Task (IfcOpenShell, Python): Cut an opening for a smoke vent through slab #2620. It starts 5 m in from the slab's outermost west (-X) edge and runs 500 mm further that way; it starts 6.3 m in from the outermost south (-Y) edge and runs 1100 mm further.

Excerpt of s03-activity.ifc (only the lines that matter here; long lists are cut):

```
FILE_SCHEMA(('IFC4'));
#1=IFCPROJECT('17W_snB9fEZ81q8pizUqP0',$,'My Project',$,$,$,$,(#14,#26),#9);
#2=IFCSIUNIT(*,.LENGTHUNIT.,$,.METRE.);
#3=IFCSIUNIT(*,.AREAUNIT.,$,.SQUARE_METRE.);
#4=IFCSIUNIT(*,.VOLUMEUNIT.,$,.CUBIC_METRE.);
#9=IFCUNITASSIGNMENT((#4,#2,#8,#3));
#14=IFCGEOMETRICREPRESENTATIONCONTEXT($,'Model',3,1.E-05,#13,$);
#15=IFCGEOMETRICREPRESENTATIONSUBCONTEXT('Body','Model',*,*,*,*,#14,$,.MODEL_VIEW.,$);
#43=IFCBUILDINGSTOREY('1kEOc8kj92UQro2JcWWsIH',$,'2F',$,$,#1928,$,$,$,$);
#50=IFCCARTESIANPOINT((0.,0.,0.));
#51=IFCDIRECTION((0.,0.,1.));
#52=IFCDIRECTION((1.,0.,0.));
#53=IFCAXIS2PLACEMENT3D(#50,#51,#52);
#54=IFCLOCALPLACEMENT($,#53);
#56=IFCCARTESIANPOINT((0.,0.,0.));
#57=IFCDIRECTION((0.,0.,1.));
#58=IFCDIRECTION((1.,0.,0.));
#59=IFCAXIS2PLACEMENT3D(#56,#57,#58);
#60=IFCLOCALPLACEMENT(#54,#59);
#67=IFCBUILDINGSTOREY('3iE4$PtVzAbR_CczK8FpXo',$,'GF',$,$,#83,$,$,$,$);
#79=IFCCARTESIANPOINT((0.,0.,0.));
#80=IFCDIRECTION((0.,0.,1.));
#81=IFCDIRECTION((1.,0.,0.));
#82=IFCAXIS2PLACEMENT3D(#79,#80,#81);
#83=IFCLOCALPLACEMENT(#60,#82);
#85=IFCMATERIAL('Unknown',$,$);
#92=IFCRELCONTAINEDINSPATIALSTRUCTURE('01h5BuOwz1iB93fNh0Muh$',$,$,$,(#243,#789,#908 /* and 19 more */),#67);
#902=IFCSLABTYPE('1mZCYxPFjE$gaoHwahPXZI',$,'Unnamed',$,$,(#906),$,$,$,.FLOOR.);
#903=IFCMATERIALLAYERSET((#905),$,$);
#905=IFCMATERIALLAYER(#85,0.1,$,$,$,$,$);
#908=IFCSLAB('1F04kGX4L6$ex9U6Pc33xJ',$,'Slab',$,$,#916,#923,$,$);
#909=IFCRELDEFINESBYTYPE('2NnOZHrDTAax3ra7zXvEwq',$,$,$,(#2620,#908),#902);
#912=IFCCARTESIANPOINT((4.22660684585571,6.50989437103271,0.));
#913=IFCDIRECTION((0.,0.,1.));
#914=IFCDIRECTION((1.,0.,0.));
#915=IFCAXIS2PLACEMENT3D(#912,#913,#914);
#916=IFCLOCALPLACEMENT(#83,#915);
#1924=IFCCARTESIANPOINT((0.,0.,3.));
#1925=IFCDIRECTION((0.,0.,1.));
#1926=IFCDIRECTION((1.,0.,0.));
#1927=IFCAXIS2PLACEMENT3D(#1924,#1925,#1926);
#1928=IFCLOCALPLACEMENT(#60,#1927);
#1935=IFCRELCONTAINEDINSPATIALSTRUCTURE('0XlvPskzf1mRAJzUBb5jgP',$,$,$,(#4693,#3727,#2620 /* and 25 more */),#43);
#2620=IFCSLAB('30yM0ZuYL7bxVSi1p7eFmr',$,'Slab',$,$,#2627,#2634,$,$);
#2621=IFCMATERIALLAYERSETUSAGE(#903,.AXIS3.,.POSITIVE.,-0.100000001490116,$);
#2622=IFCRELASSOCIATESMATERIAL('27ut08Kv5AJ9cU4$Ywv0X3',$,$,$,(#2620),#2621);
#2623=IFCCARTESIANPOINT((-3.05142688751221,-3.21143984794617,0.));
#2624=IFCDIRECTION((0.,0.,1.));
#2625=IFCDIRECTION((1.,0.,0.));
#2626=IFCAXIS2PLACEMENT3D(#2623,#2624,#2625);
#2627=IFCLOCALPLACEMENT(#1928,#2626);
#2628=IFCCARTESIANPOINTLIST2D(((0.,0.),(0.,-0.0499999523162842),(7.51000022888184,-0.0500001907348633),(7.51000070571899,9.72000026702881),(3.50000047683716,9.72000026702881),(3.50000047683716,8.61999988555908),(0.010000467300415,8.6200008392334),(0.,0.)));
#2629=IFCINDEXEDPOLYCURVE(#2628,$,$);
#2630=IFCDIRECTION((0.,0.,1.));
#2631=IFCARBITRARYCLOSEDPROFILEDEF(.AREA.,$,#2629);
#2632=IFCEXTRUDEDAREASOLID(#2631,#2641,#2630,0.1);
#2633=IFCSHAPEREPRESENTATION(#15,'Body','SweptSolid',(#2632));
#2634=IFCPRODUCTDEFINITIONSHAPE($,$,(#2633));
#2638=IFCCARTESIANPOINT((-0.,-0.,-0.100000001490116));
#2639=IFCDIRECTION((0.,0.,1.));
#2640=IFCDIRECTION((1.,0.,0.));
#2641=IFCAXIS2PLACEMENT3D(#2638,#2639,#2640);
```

```python
import numpy as np
import ifcopenshell
import ifcopenshell.api.feature
import ifcopenshell.api.geometry
import ifcopenshell.api.root
import ifcopenshell.geom
import ifcopenshell.util.placement
import ifcopenshell.util.representation
import ifcopenshell.util.shape
import ifcopenshell.util.unit

model = ifcopenshell.open("s03-activity.ifc")
unit_scale = ifcopenshell.util.unit.calculate_unit_scale(model)
settings = ifcopenshell.geom.settings()


def volume(element):
    """Net volume in cubic metres, openings subtracted."""
    shape = ifcopenshell.geom.create_shape(settings, element)
    return ifcopenshell.util.shape.get_volume(shape.geometry)


slab = model.by_guid("30yM0ZuYL7bxVSi1p7eFmr")
before = volume(slab)

# Extent in the slab's own axes, in metres. The edges named are its -X and -Y sides.
slab_shape = ifcopenshell.geom.create_shape(settings, slab)
vertices = ifcopenshell.util.shape.get_vertices(slab_shape.geometry)
x_min, y_min, bottom = vertices.min(axis=0)
top = vertices[:, 2].max()

opening = ifcopenshell.api.root.create_entity(model, ifc_class="IfcOpeningElement", name="Smoke vent opening", predefined_type="OPENING")
context = ifcopenshell.util.representation.get_context(model, "Model", "Body", "MODEL_VIEW")
width, depth = 0.5, 1.1
outline = [(0.0, 0.0), (width, 0.0), (width, depth), (0.0, depth), (0.0, 0.0)]
# Overshoot both faces by 50 mm so the cut is clean.
shape = ifcopenshell.api.geometry.add_slab_representation(
    model, context=context, depth=top - bottom + 0.1, polyline=outline
)
ifcopenshell.api.geometry.assign_representation(model, product=opening, representation=shape)

matrix = ifcopenshell.util.placement.get_local_placement(slab.ObjectPlacement)
matrix[:, 3] = matrix @ np.append(np.array([x_min + 5, y_min + 6.3, bottom - 0.05]) / unit_scale, 1.0)
ifcopenshell.api.geometry.edit_object_placement(model, product=opening, matrix=matrix, is_si=False)
ifcopenshell.api.feature.add_feature(model, feature=opening, element=slab)

after = volume(slab)

print(f"slab volume {before:.3f} -> {after:.3f} m3")

model.write("s03-activity_edited.ifc")
```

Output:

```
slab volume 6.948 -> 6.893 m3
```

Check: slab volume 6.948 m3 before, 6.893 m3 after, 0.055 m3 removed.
